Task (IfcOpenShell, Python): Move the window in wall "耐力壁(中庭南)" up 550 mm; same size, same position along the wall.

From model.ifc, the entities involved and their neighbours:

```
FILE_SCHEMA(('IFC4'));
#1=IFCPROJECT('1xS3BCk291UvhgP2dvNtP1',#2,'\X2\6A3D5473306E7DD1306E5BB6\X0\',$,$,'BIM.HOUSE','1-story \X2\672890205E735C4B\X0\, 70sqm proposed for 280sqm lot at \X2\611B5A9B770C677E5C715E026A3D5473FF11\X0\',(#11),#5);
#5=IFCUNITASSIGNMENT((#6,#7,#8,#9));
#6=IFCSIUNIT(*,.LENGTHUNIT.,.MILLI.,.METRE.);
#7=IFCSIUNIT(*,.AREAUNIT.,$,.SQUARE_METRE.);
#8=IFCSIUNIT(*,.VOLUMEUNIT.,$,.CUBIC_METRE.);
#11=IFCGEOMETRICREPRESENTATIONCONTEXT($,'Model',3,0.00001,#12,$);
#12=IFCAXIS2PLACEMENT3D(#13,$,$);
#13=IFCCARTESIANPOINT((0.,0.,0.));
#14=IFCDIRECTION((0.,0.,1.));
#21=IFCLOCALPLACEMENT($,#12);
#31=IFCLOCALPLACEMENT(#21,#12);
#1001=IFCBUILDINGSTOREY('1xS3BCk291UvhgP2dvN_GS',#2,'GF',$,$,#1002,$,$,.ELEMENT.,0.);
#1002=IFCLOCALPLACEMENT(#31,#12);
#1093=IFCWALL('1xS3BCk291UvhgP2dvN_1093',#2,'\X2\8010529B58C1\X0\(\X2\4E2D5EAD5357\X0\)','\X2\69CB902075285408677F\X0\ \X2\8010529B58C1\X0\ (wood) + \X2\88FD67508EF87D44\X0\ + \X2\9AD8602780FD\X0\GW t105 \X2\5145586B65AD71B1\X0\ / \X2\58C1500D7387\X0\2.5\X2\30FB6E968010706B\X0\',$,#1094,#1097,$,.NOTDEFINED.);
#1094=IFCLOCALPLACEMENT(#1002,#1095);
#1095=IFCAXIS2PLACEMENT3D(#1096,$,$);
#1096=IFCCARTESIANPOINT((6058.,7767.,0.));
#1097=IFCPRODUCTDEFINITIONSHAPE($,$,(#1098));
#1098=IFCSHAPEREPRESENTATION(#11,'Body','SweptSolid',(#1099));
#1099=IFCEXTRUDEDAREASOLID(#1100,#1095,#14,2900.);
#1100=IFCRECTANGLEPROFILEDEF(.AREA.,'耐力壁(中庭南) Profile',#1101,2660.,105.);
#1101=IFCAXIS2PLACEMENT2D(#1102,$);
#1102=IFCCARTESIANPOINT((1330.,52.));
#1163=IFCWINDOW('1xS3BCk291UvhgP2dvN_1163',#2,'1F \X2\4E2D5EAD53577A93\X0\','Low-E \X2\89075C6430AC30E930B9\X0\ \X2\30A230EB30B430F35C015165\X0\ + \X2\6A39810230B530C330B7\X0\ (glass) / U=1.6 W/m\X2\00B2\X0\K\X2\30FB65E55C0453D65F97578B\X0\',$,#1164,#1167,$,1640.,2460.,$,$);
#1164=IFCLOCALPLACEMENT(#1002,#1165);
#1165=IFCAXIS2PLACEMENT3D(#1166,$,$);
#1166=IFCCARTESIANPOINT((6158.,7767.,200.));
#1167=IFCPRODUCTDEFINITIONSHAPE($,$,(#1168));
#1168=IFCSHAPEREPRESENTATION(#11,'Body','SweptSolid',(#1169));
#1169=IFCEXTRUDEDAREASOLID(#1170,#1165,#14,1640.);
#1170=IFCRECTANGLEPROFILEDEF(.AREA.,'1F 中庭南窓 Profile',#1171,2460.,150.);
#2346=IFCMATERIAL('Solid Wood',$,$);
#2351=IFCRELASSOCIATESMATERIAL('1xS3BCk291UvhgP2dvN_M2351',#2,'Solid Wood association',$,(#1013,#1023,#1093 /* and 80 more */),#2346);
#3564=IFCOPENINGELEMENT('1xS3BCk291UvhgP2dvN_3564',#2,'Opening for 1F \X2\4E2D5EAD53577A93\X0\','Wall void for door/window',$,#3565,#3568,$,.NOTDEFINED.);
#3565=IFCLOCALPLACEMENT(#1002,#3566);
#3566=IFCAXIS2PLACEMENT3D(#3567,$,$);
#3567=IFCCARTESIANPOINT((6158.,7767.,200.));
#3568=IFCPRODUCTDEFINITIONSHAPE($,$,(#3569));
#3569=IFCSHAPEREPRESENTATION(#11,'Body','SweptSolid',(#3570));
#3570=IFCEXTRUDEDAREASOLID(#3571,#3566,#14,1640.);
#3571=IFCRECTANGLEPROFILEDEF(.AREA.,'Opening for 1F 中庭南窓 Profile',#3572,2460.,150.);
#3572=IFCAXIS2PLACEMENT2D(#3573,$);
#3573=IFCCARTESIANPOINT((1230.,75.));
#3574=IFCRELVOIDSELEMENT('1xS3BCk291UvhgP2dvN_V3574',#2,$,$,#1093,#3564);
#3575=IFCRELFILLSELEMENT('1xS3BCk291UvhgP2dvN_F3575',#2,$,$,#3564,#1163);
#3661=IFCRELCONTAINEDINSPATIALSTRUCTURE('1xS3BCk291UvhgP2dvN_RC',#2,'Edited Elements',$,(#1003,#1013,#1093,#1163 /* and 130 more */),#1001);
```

```python
import numpy as np
import ifcopenshell
import ifcopenshell.api.geometry
import ifcopenshell.util.placement
import ifcopenshell.util.unit

model = ifcopenshell.open("model.ifc")
unit_scale = ifcopenshell.util.unit.calculate_unit_scale(model)

window = model.by_guid("1xS3BCk291UvhgP2dvN_1163")
opening = window.FillsVoids[0].RelatingOpeningElement
dz = 0.55 / unit_scale

shift = np.array([0.0, 0.0, dz])
# The window is not placed relative to its opening, so move both.
for product in (opening, window):
    matrix = ifcopenshell.util.placement.get_local_placement(product.ObjectPlacement)
    matrix[:3, 3] += shift
    ifcopenshell.api.geometry.edit_object_placement(model, product=product, matrix=matrix, is_si=False)

print(f"moved by {dz * unit_scale:+.3f} m")

model.write("model_updated.ifc")
```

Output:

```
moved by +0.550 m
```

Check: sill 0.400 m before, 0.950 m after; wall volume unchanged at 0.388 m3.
